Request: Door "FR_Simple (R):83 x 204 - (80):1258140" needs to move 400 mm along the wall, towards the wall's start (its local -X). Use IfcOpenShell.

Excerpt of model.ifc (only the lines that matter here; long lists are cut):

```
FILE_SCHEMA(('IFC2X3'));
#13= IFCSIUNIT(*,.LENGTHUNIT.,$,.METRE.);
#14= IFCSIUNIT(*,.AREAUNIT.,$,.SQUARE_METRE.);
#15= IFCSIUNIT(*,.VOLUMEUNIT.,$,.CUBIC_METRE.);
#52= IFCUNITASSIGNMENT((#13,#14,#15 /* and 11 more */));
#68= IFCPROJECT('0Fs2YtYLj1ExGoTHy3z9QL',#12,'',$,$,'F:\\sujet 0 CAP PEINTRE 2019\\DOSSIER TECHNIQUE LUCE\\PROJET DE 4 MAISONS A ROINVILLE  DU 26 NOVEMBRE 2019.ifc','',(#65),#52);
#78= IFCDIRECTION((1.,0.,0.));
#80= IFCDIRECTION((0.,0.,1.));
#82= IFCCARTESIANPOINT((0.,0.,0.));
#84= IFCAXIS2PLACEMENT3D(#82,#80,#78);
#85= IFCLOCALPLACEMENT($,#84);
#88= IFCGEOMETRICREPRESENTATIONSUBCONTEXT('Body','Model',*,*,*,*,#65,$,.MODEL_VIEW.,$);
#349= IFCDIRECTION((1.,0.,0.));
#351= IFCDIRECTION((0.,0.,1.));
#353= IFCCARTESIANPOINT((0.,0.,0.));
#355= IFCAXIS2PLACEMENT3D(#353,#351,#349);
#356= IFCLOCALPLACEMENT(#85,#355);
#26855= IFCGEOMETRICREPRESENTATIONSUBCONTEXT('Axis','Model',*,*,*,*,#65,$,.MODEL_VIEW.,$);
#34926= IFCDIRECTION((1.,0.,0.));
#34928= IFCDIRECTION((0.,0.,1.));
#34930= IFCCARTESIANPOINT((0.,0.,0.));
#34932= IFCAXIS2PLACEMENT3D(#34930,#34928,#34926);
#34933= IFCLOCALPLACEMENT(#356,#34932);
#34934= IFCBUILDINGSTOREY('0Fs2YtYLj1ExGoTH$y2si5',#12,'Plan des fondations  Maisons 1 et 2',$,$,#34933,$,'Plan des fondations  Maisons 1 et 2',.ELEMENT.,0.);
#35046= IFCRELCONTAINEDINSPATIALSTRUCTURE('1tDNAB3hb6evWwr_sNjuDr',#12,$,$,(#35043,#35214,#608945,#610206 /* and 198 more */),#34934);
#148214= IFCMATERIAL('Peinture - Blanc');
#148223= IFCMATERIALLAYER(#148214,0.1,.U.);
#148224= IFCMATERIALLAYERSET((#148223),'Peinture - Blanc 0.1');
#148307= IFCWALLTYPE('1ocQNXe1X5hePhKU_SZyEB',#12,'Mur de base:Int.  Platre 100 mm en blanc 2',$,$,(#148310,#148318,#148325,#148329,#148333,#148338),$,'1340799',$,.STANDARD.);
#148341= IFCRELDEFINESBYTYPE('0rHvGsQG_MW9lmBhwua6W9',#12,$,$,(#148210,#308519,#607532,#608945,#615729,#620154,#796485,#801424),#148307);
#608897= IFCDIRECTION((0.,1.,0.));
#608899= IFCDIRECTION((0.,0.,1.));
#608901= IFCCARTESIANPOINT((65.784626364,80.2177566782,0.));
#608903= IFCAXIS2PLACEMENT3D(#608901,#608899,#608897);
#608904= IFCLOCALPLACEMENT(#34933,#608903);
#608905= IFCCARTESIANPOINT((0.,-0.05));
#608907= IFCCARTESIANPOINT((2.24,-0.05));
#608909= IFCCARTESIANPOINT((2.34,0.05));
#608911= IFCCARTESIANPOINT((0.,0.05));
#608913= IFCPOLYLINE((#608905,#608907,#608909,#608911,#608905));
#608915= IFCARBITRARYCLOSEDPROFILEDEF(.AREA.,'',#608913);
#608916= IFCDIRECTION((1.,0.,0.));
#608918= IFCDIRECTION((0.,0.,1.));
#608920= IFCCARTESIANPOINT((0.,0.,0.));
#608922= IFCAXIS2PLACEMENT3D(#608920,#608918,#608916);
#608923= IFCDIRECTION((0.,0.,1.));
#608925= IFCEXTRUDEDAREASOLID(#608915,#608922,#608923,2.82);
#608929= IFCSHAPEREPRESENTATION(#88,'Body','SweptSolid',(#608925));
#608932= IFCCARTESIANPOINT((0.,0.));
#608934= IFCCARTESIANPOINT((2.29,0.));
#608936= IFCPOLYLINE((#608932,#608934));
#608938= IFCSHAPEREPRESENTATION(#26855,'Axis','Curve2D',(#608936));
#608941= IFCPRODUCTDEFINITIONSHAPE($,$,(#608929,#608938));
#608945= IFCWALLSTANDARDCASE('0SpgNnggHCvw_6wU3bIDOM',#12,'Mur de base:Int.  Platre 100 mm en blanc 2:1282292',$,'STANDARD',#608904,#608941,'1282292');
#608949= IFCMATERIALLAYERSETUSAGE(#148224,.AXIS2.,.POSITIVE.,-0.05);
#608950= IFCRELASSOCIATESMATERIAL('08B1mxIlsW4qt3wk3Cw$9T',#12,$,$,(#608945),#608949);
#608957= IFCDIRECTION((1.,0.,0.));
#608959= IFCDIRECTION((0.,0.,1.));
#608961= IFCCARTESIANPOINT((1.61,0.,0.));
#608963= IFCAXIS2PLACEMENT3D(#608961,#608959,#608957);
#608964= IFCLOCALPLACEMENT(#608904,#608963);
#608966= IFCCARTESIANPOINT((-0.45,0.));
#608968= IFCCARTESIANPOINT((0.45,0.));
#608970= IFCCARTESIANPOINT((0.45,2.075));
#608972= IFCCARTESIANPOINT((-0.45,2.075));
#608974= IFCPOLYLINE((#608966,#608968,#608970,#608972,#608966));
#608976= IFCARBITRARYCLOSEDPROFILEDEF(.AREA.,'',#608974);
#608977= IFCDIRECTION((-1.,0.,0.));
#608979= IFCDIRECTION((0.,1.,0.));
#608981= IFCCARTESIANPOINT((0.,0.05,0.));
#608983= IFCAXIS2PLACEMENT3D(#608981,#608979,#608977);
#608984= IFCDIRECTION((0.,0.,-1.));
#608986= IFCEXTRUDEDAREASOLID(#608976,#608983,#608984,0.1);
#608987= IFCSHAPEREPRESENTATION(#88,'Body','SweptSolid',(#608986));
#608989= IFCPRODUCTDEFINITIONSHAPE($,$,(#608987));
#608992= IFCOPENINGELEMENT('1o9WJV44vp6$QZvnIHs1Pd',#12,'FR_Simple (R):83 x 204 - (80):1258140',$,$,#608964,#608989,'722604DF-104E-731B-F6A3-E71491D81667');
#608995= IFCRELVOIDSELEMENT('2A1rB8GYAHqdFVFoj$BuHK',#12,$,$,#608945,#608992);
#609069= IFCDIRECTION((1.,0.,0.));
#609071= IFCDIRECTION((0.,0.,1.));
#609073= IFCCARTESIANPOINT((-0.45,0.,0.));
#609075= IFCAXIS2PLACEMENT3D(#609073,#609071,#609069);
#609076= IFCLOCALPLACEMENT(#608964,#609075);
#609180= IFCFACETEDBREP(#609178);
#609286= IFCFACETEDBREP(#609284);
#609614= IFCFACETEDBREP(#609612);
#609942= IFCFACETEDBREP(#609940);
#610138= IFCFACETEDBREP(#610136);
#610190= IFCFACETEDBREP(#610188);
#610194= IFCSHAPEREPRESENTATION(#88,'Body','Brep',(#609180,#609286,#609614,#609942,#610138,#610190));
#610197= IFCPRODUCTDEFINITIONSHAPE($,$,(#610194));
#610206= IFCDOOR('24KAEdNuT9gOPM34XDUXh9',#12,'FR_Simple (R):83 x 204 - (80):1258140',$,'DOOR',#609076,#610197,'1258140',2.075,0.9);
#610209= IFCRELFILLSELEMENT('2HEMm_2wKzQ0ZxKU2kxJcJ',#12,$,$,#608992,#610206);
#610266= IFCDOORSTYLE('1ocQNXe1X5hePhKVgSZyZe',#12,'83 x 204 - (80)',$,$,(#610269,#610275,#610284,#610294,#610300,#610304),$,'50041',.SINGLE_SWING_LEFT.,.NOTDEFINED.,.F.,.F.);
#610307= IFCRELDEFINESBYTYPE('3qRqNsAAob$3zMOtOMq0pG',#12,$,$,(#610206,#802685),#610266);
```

```python
import ifcopenshell
import ifcopenshell.api.geometry
import ifcopenshell.util.placement
import ifcopenshell.util.unit

model = ifcopenshell.open("model.ifc")
unit_scale = ifcopenshell.util.unit.calculate_unit_scale(model)

door = model.by_guid("24KAEdNuT9gOPM34XDUXh9")
opening = door.FillsVoids[0].RelatingOpeningElement
wall = opening.VoidsElements[0].RelatingBuildingElement

wall_matrix = ifcopenshell.util.placement.get_local_placement(wall.ObjectPlacement)
shift = wall_matrix[:3, 0] * -0.4 / unit_scale
before = ifcopenshell.util.placement.get_local_placement(door.ObjectPlacement)[:3, 3].copy()

# The door is placed relative to its opening, so it follows when the opening moves.
matrix = ifcopenshell.util.placement.get_local_placement(opening.ObjectPlacement)
matrix[:3, 3] += shift
ifcopenshell.api.geometry.edit_object_placement(
    model, product=opening, matrix=matrix, is_si=False, should_transform_children=True
)

after = ifcopenshell.util.placement.get_local_placement(door.ObjectPlacement)[:3, 3]
print("door moved by", (after - before).round(3) + 0.0)

model.write("model-out.ifc")
```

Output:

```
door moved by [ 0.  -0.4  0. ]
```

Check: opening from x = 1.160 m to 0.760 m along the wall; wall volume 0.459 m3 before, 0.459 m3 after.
